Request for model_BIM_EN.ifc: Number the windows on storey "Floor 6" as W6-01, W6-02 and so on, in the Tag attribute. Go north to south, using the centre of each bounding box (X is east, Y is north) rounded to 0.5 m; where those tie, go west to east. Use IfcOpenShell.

First a look at what the model holds.

```python
import ifcopenshell
import ifcopenshell.util.element
import ifcopenshell.util.placement

model = ifcopenshell.open("model_BIM_EN.ifc")
print(model.schema)
storey = next(s for s in model.by_type("IfcBuildingStorey") if s.Name == "Floor 6")
windows = [e for e in ifcopenshell.util.element.get_decomposition(storey) if e.is_a("IfcWindow")]
for e in sorted(windows, key=lambda e: e.id()):
    origin = ifcopenshell.util.placement.get_local_placement(e.ObjectPlacement)[:3, 3]
    print(e.id(), e.Tag, e.Name, origin.round(2) + 0.0, sep=" | ")
```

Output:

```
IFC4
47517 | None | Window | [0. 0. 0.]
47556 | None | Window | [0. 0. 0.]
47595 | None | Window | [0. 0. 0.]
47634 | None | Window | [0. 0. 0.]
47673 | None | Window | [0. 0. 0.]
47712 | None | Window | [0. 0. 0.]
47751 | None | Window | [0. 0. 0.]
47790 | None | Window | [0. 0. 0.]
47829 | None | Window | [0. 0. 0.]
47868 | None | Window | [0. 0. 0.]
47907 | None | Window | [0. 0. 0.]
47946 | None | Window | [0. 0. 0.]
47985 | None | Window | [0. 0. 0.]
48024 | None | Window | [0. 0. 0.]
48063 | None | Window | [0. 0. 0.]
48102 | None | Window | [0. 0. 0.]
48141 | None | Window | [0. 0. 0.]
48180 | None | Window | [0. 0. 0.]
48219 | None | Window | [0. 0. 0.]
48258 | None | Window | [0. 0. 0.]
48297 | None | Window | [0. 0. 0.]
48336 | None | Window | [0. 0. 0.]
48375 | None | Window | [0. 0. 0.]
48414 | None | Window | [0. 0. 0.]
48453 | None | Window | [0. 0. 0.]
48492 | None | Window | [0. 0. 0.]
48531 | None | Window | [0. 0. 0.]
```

```python
import ifcopenshell
import ifcopenshell.geom
import ifcopenshell.util.element
import ifcopenshell.util.shape

model = ifcopenshell.open("model_BIM_EN.ifc")
settings = ifcopenshell.geom.settings()
settings.set("use-world-coords", True)


def centre(element):
    shape = ifcopenshell.geom.create_shape(settings, element)
    return ifcopenshell.util.shape.get_bbox_centroid(shape.geometry)


storey = next(s for s in model.by_type("IfcBuildingStorey") if s.Name == "Floor 6")
windows = [e for e in ifcopenshell.util.element.get_decomposition(storey) if e.is_a("IfcWindow")]

# Insertion points can sit at a corner or the storey origin, so sort by the geometry (in metres).
centres = {e: centre(e) for e in windows}
windows.sort(key=lambda e: (-round(centres[e][1] / 0.5), centres[e][0]))

for i, e in enumerate(windows, start=1):
    number = f"W6-{i:02d}"
    e.Tag = number
    print(e.id(), number)

model.write("model_BIM_EN_edited.ifc")
```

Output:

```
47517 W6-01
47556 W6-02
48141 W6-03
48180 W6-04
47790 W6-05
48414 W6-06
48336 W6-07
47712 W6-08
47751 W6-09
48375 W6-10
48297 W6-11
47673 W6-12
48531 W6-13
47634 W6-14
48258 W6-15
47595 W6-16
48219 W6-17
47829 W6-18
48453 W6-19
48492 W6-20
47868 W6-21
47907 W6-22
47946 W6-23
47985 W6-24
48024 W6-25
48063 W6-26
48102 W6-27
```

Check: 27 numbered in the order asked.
